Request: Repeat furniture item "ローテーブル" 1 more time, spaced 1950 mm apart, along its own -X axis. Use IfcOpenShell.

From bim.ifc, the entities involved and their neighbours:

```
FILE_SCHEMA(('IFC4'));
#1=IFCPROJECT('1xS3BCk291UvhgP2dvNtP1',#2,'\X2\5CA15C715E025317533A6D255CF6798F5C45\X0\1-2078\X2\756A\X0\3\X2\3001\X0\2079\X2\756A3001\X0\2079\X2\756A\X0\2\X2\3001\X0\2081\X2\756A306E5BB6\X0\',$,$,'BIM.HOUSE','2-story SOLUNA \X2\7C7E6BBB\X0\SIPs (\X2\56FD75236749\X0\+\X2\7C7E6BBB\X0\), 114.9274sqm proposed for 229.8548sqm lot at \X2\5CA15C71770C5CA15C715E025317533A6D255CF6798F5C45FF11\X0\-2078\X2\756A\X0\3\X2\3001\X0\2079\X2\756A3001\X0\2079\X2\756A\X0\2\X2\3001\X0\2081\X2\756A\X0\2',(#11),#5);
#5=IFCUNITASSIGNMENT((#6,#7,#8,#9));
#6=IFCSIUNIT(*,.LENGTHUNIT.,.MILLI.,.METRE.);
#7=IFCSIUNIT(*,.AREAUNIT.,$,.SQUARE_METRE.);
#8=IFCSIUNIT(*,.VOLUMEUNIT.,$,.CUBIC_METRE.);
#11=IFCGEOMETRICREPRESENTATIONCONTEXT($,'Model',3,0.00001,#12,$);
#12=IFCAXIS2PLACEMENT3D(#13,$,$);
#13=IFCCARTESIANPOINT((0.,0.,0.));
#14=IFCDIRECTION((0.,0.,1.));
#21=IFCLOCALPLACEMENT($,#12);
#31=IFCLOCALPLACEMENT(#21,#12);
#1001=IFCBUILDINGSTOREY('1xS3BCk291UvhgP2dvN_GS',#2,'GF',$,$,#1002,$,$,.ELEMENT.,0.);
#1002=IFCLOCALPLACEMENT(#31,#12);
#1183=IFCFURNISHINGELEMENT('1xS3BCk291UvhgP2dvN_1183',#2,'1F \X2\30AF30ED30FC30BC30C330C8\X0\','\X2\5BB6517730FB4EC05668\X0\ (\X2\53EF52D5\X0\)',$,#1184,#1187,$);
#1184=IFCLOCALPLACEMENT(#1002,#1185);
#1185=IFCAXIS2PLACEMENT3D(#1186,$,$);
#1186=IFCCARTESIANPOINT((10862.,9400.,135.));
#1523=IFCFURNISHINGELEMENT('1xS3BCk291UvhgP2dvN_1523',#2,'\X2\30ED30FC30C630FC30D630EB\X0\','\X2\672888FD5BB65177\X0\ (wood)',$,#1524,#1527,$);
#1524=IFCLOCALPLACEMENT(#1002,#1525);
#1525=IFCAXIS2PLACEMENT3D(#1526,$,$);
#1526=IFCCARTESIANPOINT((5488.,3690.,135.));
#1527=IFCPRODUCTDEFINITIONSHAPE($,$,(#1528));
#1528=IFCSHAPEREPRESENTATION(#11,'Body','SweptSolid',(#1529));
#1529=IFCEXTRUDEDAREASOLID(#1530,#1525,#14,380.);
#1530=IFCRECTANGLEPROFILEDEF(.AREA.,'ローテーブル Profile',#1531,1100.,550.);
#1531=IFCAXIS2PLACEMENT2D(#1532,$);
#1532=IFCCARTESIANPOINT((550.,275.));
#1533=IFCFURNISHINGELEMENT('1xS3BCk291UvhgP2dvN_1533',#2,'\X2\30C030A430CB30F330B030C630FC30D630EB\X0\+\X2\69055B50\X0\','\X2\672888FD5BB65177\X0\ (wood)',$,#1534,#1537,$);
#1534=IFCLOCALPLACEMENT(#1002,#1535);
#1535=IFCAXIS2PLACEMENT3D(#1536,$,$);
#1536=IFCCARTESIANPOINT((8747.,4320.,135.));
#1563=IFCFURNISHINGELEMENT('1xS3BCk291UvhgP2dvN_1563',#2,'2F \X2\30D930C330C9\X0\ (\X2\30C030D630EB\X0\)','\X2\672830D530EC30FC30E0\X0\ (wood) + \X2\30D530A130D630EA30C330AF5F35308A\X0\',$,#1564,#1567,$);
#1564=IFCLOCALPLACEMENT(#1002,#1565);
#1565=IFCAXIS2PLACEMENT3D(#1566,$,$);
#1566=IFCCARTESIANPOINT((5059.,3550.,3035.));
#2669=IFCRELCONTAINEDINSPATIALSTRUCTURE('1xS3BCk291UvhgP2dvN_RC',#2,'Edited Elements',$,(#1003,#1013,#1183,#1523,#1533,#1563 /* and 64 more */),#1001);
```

```python
import ifcopenshell
import ifcopenshell.api.geometry
import ifcopenshell.api.root
import ifcopenshell.util.element
import ifcopenshell.util.placement
import ifcopenshell.util.unit

model = ifcopenshell.open("bim.ifc")
unit_scale = ifcopenshell.util.unit.calculate_unit_scale(model)


def reuse_history(source, copy):
    """copy_class also copies each property set's owner history, people and application; keep the originals."""
    for rel in copy.IsDefinedBy:
        if rel.is_a("IfcRelDefinesByProperties") and (history := rel.RelatingPropertyDefinition.OwnerHistory):
            rel.RelatingPropertyDefinition.OwnerHistory = source.OwnerHistory
            ifcopenshell.util.element.remove_deep2(model, history)


source = model.by_id(1523)
base = ifcopenshell.util.placement.get_local_placement(source.ObjectPlacement)
step = -base[:3, 0] * 1.95 / unit_scale

for i in range(1, 2):
    copy = ifcopenshell.api.root.copy_class(model, product=source)
    copy.Representation = ifcopenshell.util.element.copy_deep(
        model, source.Representation, exclude=["IfcGeometricRepresentationContext", "IfcRepresentationMap"]
    )
    reuse_history(source, copy)
    matrix = base.copy()
    matrix[:3, 3] += i * step
    print("added at", matrix[:3, 3].round(3) + 0.0)
    ifcopenshell.api.geometry.edit_object_placement(model, product=copy, matrix=matrix, is_si=False)

model.write("bim_v2.ifc")
```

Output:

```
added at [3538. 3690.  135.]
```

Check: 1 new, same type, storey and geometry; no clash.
